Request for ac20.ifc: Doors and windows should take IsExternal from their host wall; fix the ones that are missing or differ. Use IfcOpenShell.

First a look at what the model holds.

```python
import ifcopenshell
import ifcopenshell.util.element

model = ifcopenshell.open("ac20.ifc")
print(model.schema)
seen = {}
for e in model.by_type("IfcDoor") + model.by_type("IfcWindow"):
    if not e.FillsVoids:
        continue
    host = e.FillsVoids[0].RelatingOpeningElement.VoidsElements[0].RelatingBuildingElement
    own = ifcopenshell.util.element.get_pset(e, f"Pset_{e.is_a()[3:].removesuffix('StandardCase')}Common", "IsExternal")
    wall = ifcopenshell.util.element.get_pset(host, "Pset_WallCommon", "IsExternal")
    seen[e.is_a(), own, wall] = seen.get((e.is_a(), own, wall), 0) + 1
for (cls, own, wall), count in sorted(seen.items(), key=str):
    print(count, cls, "IsExternal:", own, "| host wall:", wall)
```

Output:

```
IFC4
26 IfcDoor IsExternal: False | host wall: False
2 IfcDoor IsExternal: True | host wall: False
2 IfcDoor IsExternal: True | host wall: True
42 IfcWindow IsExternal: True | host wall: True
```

```python
import ifcopenshell
import ifcopenshell.api.pset
import ifcopenshell.util.element

model = ifcopenshell.open("ac20.ifc")

count = 0
for ifc_class, pset_name in (("IfcDoor", "Pset_DoorCommon"), ("IfcWindow", "Pset_WindowCommon")):
    for e in model.by_type(ifc_class):
        if not e.FillsVoids:
            continue
        host = e.FillsVoids[0].RelatingOpeningElement.VoidsElements[0].RelatingBuildingElement
        external = ifcopenshell.util.element.get_pset(host, "Pset_WallCommon", "IsExternal")
        if external is None or ifcopenshell.util.element.get_pset(e, pset_name, "IsExternal") == external:
            continue
        pset = ifcopenshell.api.pset.add_pset(model, product=e, name=pset_name)
        ifcopenshell.api.pset.edit_pset(model, pset=pset, properties={"IsExternal": external})
        count += 1

print(count, "updated")

model.write("ac20_updated.ifc")
```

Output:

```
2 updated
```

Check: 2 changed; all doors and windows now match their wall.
